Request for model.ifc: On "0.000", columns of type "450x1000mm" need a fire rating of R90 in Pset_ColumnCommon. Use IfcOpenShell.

First a look at what the model holds.

```python
import ifcopenshell
import ifcopenshell.util.element

model = ifcopenshell.open("model.ifc")
print(model.schema)
storey = next(s for s in model.by_type("IfcBuildingStorey") if s.Name == "0.000")
columns = [e for e in ifcopenshell.util.element.get_decomposition(storey) if e.is_a("IfcColumn")]
seen = {}
for e in columns:
    element_type = ifcopenshell.util.element.get_type(e)
    key = (element_type.Name if element_type != e and element_type else None, ifcopenshell.util.element.get_pset(e, "Pset_ColumnCommon", "FireRating"))
    seen[key] = seen.get(key, 0) + 1
for (name, value), count in sorted(seen.items(), key=str):
    print(count, "x", name, "|", value)
```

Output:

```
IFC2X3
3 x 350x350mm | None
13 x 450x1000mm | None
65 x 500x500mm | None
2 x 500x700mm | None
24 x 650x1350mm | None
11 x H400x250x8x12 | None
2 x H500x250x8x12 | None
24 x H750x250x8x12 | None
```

```python
import ifcopenshell
import ifcopenshell.api.pset
import ifcopenshell.util.element

model = ifcopenshell.open("model.ifc")

storey = next(s for s in model.by_type("IfcBuildingStorey") if s.Name == "0.000")
columns = [e for e in ifcopenshell.util.element.get_decomposition(storey) if e.is_a("IfcColumn")]

count = 0
for e in columns:
    element_type = ifcopenshell.util.element.get_type(e)
    if element_type in (None, e) or element_type.Name != "450x1000mm":
        continue
    # add_pset returns the element's existing set when there is one.
    pset = ifcopenshell.api.pset.add_pset(model, product=e, name="Pset_ColumnCommon")
    ifcopenshell.api.pset.edit_pset(model, pset=pset, properties={"FireRating": "R90"})
    count += 1

print(count, "columns updated")

model.write("model_rev.ifc")
```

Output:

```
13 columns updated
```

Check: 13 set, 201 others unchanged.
